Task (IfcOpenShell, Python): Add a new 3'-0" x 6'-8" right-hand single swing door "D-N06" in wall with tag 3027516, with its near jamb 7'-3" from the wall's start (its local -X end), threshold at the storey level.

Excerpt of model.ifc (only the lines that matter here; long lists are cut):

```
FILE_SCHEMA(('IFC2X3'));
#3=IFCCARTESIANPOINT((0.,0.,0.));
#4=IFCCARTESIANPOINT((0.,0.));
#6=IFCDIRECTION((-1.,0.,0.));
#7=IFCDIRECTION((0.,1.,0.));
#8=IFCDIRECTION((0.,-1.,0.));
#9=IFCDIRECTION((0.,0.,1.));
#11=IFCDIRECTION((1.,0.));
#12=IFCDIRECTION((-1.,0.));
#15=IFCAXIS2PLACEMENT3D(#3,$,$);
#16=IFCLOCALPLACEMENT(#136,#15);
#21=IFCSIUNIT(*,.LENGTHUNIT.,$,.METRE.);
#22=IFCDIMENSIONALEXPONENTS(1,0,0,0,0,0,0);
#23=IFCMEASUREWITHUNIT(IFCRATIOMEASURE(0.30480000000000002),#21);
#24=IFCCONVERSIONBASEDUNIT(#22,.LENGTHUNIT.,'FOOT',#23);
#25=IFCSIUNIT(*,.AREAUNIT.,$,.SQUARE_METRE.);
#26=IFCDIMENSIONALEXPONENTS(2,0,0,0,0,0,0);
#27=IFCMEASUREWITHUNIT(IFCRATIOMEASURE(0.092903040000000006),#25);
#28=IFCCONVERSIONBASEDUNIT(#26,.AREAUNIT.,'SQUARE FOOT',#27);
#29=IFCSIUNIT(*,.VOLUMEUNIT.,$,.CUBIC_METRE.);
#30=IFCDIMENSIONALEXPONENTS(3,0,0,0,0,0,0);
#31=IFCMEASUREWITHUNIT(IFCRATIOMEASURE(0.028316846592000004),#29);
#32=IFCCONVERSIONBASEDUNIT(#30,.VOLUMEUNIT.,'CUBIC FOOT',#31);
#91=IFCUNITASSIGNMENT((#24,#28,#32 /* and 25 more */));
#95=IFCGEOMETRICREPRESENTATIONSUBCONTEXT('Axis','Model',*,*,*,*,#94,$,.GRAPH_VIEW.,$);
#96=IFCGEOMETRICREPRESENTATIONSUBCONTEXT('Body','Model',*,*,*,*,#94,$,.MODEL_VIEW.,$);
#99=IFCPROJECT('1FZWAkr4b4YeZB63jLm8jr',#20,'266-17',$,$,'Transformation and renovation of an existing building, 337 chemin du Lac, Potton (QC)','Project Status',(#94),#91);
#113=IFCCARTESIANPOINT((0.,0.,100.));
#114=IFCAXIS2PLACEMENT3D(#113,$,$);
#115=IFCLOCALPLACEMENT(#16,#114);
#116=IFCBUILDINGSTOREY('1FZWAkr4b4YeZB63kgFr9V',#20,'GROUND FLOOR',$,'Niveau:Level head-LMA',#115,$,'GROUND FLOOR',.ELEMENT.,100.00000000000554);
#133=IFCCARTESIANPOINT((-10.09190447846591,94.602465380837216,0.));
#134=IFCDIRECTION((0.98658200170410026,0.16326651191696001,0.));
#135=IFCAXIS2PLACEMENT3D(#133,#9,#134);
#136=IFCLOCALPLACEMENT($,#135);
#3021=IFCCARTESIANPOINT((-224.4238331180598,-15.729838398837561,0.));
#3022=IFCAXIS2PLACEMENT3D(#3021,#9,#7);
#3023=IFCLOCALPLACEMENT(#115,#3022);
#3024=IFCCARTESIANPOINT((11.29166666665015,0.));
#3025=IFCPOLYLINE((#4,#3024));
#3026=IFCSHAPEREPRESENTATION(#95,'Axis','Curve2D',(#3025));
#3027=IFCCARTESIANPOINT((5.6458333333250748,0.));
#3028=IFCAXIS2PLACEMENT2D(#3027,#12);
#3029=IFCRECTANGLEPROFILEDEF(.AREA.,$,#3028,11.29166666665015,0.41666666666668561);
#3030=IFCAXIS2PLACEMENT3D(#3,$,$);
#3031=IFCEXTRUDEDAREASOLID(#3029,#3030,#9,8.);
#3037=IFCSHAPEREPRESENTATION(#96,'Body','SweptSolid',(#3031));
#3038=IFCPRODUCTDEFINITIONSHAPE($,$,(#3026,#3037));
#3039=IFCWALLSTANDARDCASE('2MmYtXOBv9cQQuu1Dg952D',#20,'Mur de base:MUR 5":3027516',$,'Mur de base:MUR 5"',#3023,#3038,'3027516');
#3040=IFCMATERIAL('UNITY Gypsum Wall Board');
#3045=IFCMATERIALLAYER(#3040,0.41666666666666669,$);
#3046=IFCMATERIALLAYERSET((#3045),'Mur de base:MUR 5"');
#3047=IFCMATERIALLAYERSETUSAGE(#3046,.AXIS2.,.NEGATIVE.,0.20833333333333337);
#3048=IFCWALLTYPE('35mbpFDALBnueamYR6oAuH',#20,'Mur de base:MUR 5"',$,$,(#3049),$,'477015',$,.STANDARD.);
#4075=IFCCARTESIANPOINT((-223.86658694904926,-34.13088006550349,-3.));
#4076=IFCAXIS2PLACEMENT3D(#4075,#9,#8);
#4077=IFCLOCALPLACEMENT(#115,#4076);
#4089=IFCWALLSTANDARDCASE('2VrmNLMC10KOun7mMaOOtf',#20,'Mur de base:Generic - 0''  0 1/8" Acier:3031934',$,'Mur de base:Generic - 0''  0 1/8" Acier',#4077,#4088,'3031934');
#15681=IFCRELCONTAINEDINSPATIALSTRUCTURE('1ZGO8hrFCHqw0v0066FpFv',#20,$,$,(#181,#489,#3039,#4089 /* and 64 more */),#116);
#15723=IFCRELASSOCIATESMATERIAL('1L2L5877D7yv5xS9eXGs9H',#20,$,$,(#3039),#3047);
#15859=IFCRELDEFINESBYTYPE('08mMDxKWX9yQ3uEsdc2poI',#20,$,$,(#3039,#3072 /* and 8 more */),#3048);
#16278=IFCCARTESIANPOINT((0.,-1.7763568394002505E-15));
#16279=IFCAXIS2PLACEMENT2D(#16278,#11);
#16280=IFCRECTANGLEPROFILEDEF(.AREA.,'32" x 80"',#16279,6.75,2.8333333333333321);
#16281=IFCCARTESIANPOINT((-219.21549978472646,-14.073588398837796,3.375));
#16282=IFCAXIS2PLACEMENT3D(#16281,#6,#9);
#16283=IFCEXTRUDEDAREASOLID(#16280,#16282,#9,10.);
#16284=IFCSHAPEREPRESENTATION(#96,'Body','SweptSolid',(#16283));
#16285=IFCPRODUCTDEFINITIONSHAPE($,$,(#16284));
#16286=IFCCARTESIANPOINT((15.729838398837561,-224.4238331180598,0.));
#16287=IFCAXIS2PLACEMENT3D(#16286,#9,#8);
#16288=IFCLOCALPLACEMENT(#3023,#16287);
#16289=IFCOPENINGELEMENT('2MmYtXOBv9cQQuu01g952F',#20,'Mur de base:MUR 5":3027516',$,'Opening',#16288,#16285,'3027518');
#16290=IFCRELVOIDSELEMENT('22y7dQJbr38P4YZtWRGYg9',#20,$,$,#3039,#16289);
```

```python
import numpy as np
import ifcopenshell
import ifcopenshell.api.feature
import ifcopenshell.api.geometry
import ifcopenshell.api.root
import ifcopenshell.api.spatial
import ifcopenshell.api.type
import ifcopenshell.geom
import ifcopenshell.util.element
import ifcopenshell.util.placement
import ifcopenshell.util.representation
import ifcopenshell.util.shape
import ifcopenshell.util.unit

model = ifcopenshell.open("model.ifc")
unit_scale = ifcopenshell.util.unit.calculate_unit_scale(model)
settings = ifcopenshell.geom.settings()


def volume(element):
    """Net volume in cubic metres, openings subtracted."""
    shape = ifcopenshell.geom.create_shape(settings, element)
    return ifcopenshell.util.shape.get_volume(shape.geometry)


wall = model.by_guid("2MmYtXOBv9cQQuu1Dg952D")
storey = ifcopenshell.util.element.get_container(wall, ifc_class="IfcBuildingStorey")
context = ifcopenshell.util.representation.get_context(model, "Model", "Body", "MODEL_VIEW")
before = volume(wall)

width, height, from_end, sill = 0.9144, 2.032, 2.2098, 0.0  # metres

# The wall runs along its own X axis, and the end named is its -X end.
wall_shape = ifcopenshell.geom.create_shape(settings, wall)
x, y, z = ifcopenshell.util.shape.get_vertices(wall_shape.geometry).T
start = x.min() + from_end
face, thickness = float(y.min()), float(y.max() - y.min())
wall_matrix = ifcopenshell.util.placement.get_local_placement(wall.ObjectPlacement)
level = ifcopenshell.util.placement.get_local_placement(storey.ObjectPlacement)[2, 3]


def in_wall(x, y):
    """Placement at x, y metres in the wall's axes, at sill height."""
    matrix = wall_matrix.copy()
    matrix[:, 3] = wall_matrix @ np.array([x / unit_scale, y / unit_scale, 0.0, 1.0])
    matrix[2, 3] = level + sill / unit_scale
    return matrix


# Opening: a box that overshoots both wall faces by 50 mm.
opening = ifcopenshell.api.root.create_entity(model, ifc_class="IfcOpeningElement")
box = ifcopenshell.api.geometry.add_wall_representation(
    model, context=context, length=width, height=height, thickness=thickness + 0.1
)
ifcopenshell.api.geometry.assign_representation(model, product=opening, representation=box)
ifcopenshell.api.geometry.edit_object_placement(model, product=opening, matrix=in_wall(start, face - 0.05), is_si=False)
ifcopenshell.api.feature.add_feature(model, feature=opening, element=wall)

door = ifcopenshell.api.root.create_entity(model, ifc_class="IfcDoor", name="D-N06")
door.OverallWidth, door.OverallHeight = width / unit_scale, height / unit_scale
body = ifcopenshell.api.geometry.add_door_representation(
    model,
    context=context,
    overall_width=door.OverallWidth,
    overall_height=door.OverallHeight,
    operation_type="SINGLE_SWING_RIGHT",
    lining_properties={"LiningDepth": thickness / unit_scale, "ThresholdDepth": thickness / unit_scale},
)
ifcopenshell.api.geometry.assign_representation(model, product=door, representation=body)
ifcopenshell.api.spatial.assign_container(model, products=[door], relating_structure=storey)
fills = ifcopenshell.api.feature.add_filling(model, opening=opening, element=door)
fills.OwnerHistory = door.OwnerHistory  # required in IFC2X3

# IFC2X3 keeps the operation on the door style.
style = ifcopenshell.api.root.create_entity(model, ifc_class="IfcDoorStyle", name="D-N06")
style.OperationType, style.ConstructionType = "SINGLE_SWING_RIGHT", "NOTDEFINED"
style.ParameterTakesPrecedence = style.Sizeable = False
ifcopenshell.api.type.assign_type(model, related_objects=[door], relating_type=style)

# The lining spans the wall, so the door starts at the wall face.
ifcopenshell.api.geometry.edit_object_placement(model, product=door, matrix=in_wall(start, face), is_si=False)

after = volume(wall)

print(f"wall volume {before:.3f} -> {after:.3f} m3")

model.write("model_rev.ifc")
```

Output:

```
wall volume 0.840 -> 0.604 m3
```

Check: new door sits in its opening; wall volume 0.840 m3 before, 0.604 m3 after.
